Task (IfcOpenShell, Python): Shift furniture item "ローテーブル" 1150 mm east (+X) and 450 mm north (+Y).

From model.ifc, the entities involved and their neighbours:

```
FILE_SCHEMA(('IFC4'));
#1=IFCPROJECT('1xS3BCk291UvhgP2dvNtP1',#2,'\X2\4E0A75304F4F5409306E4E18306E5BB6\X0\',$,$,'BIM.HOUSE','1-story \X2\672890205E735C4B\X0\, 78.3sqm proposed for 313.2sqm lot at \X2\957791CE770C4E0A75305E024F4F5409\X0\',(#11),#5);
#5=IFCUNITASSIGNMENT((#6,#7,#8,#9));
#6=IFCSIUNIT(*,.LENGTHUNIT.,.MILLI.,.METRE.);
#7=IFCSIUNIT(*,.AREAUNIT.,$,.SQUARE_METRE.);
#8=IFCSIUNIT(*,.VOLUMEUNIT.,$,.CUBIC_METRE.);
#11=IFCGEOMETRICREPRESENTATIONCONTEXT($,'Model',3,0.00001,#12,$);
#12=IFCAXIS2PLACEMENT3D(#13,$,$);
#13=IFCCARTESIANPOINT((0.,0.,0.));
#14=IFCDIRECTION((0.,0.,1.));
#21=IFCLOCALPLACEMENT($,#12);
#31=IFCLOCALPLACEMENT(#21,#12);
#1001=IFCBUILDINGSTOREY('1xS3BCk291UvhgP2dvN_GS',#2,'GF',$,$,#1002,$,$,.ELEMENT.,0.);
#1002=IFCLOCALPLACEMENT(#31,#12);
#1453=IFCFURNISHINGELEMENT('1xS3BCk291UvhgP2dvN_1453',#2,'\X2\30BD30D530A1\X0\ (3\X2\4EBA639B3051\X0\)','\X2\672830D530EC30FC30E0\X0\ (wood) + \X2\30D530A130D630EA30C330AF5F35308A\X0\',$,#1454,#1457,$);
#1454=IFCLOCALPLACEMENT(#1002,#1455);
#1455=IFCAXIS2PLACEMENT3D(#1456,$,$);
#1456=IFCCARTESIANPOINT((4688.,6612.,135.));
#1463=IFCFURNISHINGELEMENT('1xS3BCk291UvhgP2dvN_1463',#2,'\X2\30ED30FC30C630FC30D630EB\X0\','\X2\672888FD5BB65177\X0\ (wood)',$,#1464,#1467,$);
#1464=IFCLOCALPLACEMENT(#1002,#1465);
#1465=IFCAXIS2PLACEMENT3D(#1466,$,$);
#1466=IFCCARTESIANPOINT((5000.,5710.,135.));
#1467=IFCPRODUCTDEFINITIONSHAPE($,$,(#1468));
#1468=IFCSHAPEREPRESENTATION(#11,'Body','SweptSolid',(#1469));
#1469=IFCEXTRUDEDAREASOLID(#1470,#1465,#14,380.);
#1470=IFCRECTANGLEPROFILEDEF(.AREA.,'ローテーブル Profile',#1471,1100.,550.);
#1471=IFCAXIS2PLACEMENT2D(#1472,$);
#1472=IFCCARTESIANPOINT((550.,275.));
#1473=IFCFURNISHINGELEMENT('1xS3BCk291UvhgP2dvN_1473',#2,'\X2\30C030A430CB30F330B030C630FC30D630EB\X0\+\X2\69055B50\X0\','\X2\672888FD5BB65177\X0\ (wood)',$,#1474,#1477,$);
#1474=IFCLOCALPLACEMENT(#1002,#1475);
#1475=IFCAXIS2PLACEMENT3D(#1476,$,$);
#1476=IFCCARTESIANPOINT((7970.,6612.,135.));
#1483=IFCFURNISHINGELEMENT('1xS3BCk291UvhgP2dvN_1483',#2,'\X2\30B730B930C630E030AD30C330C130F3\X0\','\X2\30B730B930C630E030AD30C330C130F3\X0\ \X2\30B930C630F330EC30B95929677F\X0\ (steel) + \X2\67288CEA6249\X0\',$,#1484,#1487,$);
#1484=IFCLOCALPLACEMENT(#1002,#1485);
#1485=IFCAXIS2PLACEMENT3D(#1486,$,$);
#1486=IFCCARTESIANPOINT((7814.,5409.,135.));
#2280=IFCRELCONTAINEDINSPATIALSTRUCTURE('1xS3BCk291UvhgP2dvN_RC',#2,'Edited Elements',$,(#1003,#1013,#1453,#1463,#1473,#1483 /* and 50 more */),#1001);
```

```python
import ifcopenshell
import ifcopenshell.api.geometry
import ifcopenshell.util.placement
import ifcopenshell.util.unit

model = ifcopenshell.open("model.ifc")
unit_scale = ifcopenshell.util.unit.calculate_unit_scale(model)

item = model.by_guid("1xS3BCk291UvhgP2dvN_1463")
matrix = ifcopenshell.util.placement.get_local_placement(item.ObjectPlacement)
matrix[0, 3] += 1.15 / unit_scale
matrix[1, 3] += 0.45 / unit_scale
ifcopenshell.api.geometry.edit_object_placement(model, product=item, matrix=matrix, is_si=False)

print(ifcopenshell.util.placement.get_local_placement(item.ObjectPlacement).round(3) + 0.0)

model.write("model_edited.ifc")
```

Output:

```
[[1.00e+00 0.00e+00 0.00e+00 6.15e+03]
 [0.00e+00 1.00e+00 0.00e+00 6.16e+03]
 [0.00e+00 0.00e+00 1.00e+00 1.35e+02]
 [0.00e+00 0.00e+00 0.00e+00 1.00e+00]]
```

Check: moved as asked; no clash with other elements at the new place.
